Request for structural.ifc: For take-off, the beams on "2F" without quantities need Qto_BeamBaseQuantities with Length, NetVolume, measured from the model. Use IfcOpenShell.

First a look at what the model holds.

```python
import ifcopenshell
import ifcopenshell.util.element
import ifcopenshell.util.unit

model = ifcopenshell.open("structural.ifc")
print(model.schema)
for unit_type in ("LENGTHUNIT", "AREAUNIT", "VOLUMEUNIT"):
    print(unit_type, ifcopenshell.util.unit.calculate_unit_scale(model, unit_type))
storey = next(s for s in model.by_type("IfcBuildingStorey") if s.Name == "2F")
beams = [e for e in ifcopenshell.util.element.get_decomposition(storey) if e.is_a("IfcBeam")]
for e in sorted(beams, key=lambda e: e.id()):
    print(e.id(), e.is_a(), e.Name, list(ifcopenshell.util.element.get_psets(e, qtos_only=True)), sep=" | ")
```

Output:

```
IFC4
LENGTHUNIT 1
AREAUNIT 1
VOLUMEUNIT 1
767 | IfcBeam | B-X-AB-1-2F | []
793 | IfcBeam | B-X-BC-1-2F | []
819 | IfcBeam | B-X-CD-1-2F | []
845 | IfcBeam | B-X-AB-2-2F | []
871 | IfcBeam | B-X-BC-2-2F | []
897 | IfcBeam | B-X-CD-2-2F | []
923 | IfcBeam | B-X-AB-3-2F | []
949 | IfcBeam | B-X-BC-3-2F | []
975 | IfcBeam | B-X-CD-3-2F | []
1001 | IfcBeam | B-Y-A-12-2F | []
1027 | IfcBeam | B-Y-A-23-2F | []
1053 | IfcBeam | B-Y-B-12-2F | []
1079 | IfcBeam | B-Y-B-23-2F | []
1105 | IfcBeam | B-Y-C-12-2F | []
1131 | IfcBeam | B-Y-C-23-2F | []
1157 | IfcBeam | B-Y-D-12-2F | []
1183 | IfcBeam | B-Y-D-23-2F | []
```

```python
import ifcopenshell
import ifcopenshell.api.pset
import ifcopenshell.geom
import ifcopenshell.util.element
import ifcopenshell.util.shape
import ifcopenshell.util.unit

model = ifcopenshell.open("structural.ifc")
unit_scale = ifcopenshell.util.unit.calculate_unit_scale(model)
volume_scale = ifcopenshell.util.unit.calculate_unit_scale(model, "VOLUMEUNIT")
settings = ifcopenshell.geom.settings()

storey = next(s for s in model.by_type("IfcBuildingStorey") if s.Name == "2F")
beams = [e for e in ifcopenshell.util.element.get_decomposition(storey) if e.is_a("IfcBeam")]

for e in sorted(beams, key=lambda e: e.id()):
    if ifcopenshell.util.element.get_psets(e, qtos_only=True, should_inherit=False):
        continue
    # Geometry comes back in metres, in the element's own axes.
    shape = ifcopenshell.geom.create_shape(settings, e)
    values = {
        "Length": ifcopenshell.util.shape.get_max_xyz(shape.geometry) / unit_scale,
        "NetVolume": ifcopenshell.util.shape.get_volume(shape.geometry) / volume_scale,
    }
    qto = ifcopenshell.api.pset.add_qto(model, product=e, name="Qto_BeamBaseQuantities")
    ifcopenshell.api.pset.edit_qto(model, qto=qto, properties=values)
    print(e.id(), {k: round(v, 3) for k, v in values.items()})

model.write("structural-out.ifc")
```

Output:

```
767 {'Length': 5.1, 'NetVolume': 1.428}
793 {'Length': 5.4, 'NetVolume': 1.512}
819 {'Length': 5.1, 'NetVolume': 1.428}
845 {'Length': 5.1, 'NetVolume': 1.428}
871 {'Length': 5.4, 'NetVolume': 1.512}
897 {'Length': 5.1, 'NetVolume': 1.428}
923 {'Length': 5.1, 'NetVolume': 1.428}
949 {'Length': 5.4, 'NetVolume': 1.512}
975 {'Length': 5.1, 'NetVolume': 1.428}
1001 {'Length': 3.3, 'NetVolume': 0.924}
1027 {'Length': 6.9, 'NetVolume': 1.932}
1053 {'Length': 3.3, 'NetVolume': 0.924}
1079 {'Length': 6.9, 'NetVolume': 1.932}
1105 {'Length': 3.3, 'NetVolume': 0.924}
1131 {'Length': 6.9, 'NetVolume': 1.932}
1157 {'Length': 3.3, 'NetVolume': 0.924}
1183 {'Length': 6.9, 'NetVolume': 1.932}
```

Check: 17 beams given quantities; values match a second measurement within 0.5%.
